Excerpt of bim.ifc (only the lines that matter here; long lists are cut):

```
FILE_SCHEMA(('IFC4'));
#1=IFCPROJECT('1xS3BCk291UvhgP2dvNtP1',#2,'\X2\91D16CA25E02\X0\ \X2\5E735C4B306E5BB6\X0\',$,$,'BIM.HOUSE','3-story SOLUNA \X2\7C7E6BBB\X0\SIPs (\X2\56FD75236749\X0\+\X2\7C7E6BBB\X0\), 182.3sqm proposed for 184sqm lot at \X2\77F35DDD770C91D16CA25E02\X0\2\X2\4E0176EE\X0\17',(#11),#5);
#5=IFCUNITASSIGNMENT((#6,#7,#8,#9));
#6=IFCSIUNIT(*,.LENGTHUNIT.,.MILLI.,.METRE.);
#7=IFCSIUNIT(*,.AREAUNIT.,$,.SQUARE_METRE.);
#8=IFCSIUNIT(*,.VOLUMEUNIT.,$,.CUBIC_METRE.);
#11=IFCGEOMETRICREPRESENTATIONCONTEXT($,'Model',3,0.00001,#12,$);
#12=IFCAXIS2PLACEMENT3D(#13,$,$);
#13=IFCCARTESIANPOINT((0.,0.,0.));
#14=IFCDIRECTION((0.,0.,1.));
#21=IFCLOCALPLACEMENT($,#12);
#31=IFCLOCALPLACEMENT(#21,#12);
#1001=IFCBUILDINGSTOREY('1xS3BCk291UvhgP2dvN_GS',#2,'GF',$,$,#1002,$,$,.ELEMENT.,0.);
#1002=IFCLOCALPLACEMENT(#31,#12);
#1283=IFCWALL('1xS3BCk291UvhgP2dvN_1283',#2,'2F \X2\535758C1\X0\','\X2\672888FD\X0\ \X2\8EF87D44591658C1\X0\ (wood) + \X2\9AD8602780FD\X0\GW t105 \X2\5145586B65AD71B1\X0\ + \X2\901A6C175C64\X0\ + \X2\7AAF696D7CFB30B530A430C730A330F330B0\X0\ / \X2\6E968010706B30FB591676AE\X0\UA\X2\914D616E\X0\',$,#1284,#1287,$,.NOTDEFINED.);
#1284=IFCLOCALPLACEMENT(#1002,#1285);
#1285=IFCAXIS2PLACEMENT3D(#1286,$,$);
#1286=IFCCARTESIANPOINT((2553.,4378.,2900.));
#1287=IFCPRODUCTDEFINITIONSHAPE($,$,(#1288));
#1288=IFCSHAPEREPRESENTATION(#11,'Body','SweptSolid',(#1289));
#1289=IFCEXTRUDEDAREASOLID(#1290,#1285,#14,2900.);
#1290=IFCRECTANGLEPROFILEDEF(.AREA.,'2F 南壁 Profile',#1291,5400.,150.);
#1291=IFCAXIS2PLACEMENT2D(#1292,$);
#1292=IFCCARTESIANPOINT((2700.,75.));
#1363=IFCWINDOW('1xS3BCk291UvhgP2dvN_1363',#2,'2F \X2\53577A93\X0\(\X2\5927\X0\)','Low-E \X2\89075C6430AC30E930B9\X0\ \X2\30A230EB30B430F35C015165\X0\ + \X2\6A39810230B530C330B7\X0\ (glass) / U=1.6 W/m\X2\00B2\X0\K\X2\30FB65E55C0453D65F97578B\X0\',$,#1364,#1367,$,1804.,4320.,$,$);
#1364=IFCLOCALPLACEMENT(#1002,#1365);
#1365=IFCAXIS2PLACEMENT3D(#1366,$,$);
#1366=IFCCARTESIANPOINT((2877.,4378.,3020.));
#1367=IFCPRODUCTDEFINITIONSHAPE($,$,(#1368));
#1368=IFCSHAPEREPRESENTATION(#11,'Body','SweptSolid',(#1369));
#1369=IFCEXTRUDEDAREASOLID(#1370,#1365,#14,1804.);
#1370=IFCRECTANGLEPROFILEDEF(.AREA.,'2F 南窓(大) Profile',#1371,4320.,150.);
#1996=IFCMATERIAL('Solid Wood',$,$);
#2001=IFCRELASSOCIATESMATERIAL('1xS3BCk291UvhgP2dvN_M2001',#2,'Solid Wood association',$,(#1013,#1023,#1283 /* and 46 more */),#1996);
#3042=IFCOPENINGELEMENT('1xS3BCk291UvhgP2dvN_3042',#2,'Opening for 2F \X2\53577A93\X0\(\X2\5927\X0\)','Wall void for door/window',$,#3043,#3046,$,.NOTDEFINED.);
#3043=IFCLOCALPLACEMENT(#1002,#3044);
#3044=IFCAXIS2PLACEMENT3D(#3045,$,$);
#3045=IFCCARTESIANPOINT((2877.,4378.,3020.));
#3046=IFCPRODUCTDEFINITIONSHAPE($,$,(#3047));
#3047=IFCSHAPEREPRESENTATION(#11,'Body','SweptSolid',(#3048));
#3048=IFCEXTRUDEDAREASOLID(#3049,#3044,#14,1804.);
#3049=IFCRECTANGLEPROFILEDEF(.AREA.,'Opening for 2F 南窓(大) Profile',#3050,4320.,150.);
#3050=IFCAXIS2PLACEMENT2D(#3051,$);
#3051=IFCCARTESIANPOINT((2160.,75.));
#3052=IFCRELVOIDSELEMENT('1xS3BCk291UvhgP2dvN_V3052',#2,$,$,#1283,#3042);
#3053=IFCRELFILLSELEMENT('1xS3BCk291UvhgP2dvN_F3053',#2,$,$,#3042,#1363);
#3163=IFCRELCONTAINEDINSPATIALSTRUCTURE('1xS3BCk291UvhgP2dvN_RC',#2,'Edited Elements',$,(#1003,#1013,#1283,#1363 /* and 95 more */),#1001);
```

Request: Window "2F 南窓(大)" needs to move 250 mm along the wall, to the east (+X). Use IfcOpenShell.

```python
import ifcopenshell
import ifcopenshell.api.geometry
import ifcopenshell.util.placement
import ifcopenshell.util.unit

model = ifcopenshell.open("bim.ifc")
unit_scale = ifcopenshell.util.unit.calculate_unit_scale(model)

window = model.by_id(1363)
opening = window.FillsVoids[0].RelatingOpeningElement
wall = opening.VoidsElements[0].RelatingBuildingElement

wall_matrix = ifcopenshell.util.placement.get_local_placement(wall.ObjectPlacement)
shift = wall_matrix[:3, 0] * 0.25 / unit_scale
before = ifcopenshell.util.placement.get_local_placement(window.ObjectPlacement)[:3, 3].copy()

# The window is not placed relative to its opening, so move both.
for product in (opening, window):
    matrix = ifcopenshell.util.placement.get_local_placement(product.ObjectPlacement)
    matrix[:3, 3] += shift
    ifcopenshell.api.geometry.edit_object_placement(model, product=product, matrix=matrix, is_si=False)

after = ifcopenshell.util.placement.get_local_placement(window.ObjectPlacement)[:3, 3]
print("window moved by", (after - before).round(3) + 0.0)

model.write("bim_updated.ifc")
```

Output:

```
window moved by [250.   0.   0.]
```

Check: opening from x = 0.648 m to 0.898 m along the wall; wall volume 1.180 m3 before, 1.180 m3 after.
